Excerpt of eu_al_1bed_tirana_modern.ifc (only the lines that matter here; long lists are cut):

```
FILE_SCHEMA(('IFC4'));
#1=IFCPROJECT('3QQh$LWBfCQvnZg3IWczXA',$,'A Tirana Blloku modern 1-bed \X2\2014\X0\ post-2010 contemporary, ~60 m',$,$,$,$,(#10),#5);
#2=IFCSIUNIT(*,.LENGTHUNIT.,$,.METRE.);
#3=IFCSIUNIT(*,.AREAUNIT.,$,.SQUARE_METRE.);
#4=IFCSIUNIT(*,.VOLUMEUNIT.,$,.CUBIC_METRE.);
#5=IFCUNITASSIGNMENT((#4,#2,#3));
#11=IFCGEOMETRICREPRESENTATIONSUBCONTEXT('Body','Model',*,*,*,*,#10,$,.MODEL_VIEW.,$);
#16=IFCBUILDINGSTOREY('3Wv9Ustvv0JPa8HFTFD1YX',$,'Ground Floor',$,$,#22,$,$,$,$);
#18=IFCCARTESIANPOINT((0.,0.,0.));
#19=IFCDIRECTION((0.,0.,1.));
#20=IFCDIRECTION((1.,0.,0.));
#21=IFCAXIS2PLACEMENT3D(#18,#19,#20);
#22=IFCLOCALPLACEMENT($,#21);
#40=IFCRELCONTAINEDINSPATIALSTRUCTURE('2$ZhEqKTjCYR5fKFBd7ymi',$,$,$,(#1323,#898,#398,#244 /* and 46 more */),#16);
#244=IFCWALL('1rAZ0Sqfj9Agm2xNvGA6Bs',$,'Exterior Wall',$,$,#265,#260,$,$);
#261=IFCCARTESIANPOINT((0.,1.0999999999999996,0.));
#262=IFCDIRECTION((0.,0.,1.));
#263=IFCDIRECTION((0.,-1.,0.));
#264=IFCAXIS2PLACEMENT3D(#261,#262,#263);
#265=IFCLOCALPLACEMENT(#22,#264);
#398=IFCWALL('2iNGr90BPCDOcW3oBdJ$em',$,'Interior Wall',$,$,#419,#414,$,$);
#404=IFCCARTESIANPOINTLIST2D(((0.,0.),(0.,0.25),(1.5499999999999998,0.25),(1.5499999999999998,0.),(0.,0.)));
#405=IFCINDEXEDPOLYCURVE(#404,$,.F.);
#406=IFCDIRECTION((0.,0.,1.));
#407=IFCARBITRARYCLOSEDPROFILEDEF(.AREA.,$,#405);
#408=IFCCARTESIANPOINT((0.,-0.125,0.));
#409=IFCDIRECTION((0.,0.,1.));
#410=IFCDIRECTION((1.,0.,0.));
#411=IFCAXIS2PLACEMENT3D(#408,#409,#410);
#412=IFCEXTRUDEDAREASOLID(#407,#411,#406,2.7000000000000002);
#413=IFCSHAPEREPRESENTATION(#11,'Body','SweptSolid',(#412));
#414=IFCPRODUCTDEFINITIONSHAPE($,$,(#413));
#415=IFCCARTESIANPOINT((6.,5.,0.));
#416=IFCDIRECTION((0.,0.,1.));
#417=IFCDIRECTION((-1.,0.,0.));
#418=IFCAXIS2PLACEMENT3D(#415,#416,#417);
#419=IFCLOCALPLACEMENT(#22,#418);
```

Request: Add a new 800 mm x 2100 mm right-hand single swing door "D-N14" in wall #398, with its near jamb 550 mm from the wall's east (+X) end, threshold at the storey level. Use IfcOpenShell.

```python
import numpy as np
import ifcopenshell
import ifcopenshell.api.feature
import ifcopenshell.api.geometry
import ifcopenshell.api.root
import ifcopenshell.api.spatial
import ifcopenshell.geom
import ifcopenshell.util.element
import ifcopenshell.util.placement
import ifcopenshell.util.representation
import ifcopenshell.util.shape
import ifcopenshell.util.unit

model = ifcopenshell.open("eu_al_1bed_tirana_modern.ifc")
unit_scale = ifcopenshell.util.unit.calculate_unit_scale(model)
settings = ifcopenshell.geom.settings()


def volume(element):
    """Net volume in cubic metres, openings subtracted."""
    shape = ifcopenshell.geom.create_shape(settings, element)
    return ifcopenshell.util.shape.get_volume(shape.geometry)


wall = model.by_guid("2iNGr90BPCDOcW3oBdJ$em")
storey = ifcopenshell.util.element.get_container(wall, ifc_class="IfcBuildingStorey")
context = ifcopenshell.util.representation.get_context(model, "Model", "Body", "MODEL_VIEW")
before = volume(wall)

width, height, from_end, sill = 0.8, 2.1, 0.55, 0.0  # metres

# The wall runs along its own X axis, and the end named is its -X end.
wall_shape = ifcopenshell.geom.create_shape(settings, wall)
x, y, z = ifcopenshell.util.shape.get_vertices(wall_shape.geometry).T
start = x.min() + from_end
face, thickness = float(y.min()), float(y.max() - y.min())
wall_matrix = ifcopenshell.util.placement.get_local_placement(wall.ObjectPlacement)
level = ifcopenshell.util.placement.get_local_placement(storey.ObjectPlacement)[2, 3]


def in_wall(x, y):
    """Placement at x, y metres in the wall's axes, at sill height."""
    matrix = wall_matrix.copy()
    matrix[:, 3] = wall_matrix @ np.array([x / unit_scale, y / unit_scale, 0.0, 1.0])
    matrix[2, 3] = level + sill / unit_scale
    return matrix


# Opening: a box that overshoots both wall faces by 50 mm.
opening = ifcopenshell.api.root.create_entity(model, ifc_class="IfcOpeningElement", predefined_type="OPENING")
box = ifcopenshell.api.geometry.add_wall_representation(
    model, context=context, length=width, height=height, thickness=thickness + 0.1
)
ifcopenshell.api.geometry.assign_representation(model, product=opening, representation=box)
ifcopenshell.api.geometry.edit_object_placement(model, product=opening, matrix=in_wall(start, face - 0.05), is_si=False)
ifcopenshell.api.feature.add_feature(model, feature=opening, element=wall)

door = ifcopenshell.api.root.create_entity(model, ifc_class="IfcDoor", name="D-N14", predefined_type="DOOR")
door.OverallWidth, door.OverallHeight = width / unit_scale, height / unit_scale
door.OperationType = "SINGLE_SWING_RIGHT"
body = ifcopenshell.api.geometry.add_door_representation(
    model,
    context=context,
    overall_width=door.OverallWidth,
    overall_height=door.OverallHeight,
    operation_type="SINGLE_SWING_RIGHT",
    lining_properties={"LiningDepth": thickness / unit_scale, "ThresholdDepth": thickness / unit_scale},
)
ifcopenshell.api.geometry.assign_representation(model, product=door, representation=body)
ifcopenshell.api.spatial.assign_container(model, products=[door], relating_structure=storey)
ifcopenshell.api.feature.add_filling(model, opening=opening, element=door)

# The lining spans the wall, so the door starts at the wall face.
ifcopenshell.api.geometry.edit_object_placement(model, product=door, matrix=in_wall(start, face), is_si=False)

after = volume(wall)

print(f"wall volume {before:.3f} -> {after:.3f} m3")

model.write("eu_al_1bed_tirana_modern-out.ifc")
```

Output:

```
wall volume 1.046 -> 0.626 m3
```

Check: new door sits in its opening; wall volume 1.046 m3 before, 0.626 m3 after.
